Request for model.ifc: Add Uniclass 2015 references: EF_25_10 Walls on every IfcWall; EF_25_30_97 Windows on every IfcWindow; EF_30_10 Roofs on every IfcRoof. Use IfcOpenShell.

First a look at what the model holds.

```python
import ifcopenshell

model = ifcopenshell.open("model.ifc")
print(model.schema)
print("classifications:", [c.Name for c in model.by_type("IfcClassification")])
for ifc_class in ("IfcDoor", "IfcRoof", "IfcStair", "IfcWall", "IfcWindow"):
    print(ifc_class, len(model.by_type(ifc_class)))
```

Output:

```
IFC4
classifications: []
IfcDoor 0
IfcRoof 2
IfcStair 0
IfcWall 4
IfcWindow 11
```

```python
import ifcopenshell
import ifcopenshell.api.classification

model = ifcopenshell.open("model.ifc")

system = ifcopenshell.api.classification.add_classification(model, classification="Uniclass 2015")

codes = {
    "IfcWall": ("EF_25_10", "Walls"),
    "IfcWindow": ("EF_25_30_97", "Windows"),
    "IfcRoof": ("EF_30_10", "Roofs"),
}
for ifc_class, (code, name) in codes.items():
    products = model.by_type(ifc_class)
    ifcopenshell.api.classification.add_reference(
        model, products=products, classification=system, identification=code, name=name
    )
    print(code, len(products))

model.write("model_updated.ifc")
```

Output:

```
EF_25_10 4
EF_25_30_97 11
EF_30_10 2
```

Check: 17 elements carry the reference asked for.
